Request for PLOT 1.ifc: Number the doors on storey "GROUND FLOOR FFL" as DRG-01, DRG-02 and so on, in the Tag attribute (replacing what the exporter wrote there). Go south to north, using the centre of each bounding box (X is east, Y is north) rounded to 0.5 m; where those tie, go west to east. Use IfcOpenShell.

First a look at what the model holds.

```python
import ifcopenshell
import ifcopenshell.util.element
import ifcopenshell.util.placement

model = ifcopenshell.open("PLOT 1.ifc")
print(model.schema)
storey = next(s for s in model.by_type("IfcBuildingStorey") if s.Name == "GROUND FLOOR FFL")
doors = [e for e in ifcopenshell.util.element.get_decomposition(storey) if e.is_a("IfcDoor")]
for e in sorted(doors, key=lambda e: e.id()):
    origin = ifcopenshell.util.placement.get_local_placement(e.ObjectPlacement)[:3, 3]
    print(e.id(), e.Tag, e.Name, origin.round(2) + 0.0, sep=" | ")
```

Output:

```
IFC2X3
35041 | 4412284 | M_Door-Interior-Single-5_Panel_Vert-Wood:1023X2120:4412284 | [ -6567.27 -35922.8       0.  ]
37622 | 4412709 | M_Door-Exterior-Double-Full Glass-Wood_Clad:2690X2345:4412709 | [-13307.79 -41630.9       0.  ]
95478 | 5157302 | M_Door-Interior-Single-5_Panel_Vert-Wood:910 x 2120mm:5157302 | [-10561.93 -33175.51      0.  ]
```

```python
import ifcopenshell
import ifcopenshell.geom
import ifcopenshell.util.element
import ifcopenshell.util.shape

model = ifcopenshell.open("PLOT 1.ifc")
settings = ifcopenshell.geom.settings()
settings.set("use-world-coords", True)


def centre(element):
    shape = ifcopenshell.geom.create_shape(settings, element)
    return ifcopenshell.util.shape.get_bbox_centroid(shape.geometry)


storey = next(s for s in model.by_type("IfcBuildingStorey") if s.Name == "GROUND FLOOR FFL")
doors = [e for e in ifcopenshell.util.element.get_decomposition(storey) if e.is_a("IfcDoor")]

# Insertion points can sit at a corner or the storey origin, so sort by the geometry (in metres).
centres = {e: centre(e) for e in doors}
doors.sort(key=lambda e: (round(centres[e][1] / 0.5), centres[e][0]))

for i, e in enumerate(doors, start=1):
    number = f"DRG-{i:02d}"
    e.Tag = number
    print(e.id(), number)

model.write("PLOT 1_updated.ifc")
```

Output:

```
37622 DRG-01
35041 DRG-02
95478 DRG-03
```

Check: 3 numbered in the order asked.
